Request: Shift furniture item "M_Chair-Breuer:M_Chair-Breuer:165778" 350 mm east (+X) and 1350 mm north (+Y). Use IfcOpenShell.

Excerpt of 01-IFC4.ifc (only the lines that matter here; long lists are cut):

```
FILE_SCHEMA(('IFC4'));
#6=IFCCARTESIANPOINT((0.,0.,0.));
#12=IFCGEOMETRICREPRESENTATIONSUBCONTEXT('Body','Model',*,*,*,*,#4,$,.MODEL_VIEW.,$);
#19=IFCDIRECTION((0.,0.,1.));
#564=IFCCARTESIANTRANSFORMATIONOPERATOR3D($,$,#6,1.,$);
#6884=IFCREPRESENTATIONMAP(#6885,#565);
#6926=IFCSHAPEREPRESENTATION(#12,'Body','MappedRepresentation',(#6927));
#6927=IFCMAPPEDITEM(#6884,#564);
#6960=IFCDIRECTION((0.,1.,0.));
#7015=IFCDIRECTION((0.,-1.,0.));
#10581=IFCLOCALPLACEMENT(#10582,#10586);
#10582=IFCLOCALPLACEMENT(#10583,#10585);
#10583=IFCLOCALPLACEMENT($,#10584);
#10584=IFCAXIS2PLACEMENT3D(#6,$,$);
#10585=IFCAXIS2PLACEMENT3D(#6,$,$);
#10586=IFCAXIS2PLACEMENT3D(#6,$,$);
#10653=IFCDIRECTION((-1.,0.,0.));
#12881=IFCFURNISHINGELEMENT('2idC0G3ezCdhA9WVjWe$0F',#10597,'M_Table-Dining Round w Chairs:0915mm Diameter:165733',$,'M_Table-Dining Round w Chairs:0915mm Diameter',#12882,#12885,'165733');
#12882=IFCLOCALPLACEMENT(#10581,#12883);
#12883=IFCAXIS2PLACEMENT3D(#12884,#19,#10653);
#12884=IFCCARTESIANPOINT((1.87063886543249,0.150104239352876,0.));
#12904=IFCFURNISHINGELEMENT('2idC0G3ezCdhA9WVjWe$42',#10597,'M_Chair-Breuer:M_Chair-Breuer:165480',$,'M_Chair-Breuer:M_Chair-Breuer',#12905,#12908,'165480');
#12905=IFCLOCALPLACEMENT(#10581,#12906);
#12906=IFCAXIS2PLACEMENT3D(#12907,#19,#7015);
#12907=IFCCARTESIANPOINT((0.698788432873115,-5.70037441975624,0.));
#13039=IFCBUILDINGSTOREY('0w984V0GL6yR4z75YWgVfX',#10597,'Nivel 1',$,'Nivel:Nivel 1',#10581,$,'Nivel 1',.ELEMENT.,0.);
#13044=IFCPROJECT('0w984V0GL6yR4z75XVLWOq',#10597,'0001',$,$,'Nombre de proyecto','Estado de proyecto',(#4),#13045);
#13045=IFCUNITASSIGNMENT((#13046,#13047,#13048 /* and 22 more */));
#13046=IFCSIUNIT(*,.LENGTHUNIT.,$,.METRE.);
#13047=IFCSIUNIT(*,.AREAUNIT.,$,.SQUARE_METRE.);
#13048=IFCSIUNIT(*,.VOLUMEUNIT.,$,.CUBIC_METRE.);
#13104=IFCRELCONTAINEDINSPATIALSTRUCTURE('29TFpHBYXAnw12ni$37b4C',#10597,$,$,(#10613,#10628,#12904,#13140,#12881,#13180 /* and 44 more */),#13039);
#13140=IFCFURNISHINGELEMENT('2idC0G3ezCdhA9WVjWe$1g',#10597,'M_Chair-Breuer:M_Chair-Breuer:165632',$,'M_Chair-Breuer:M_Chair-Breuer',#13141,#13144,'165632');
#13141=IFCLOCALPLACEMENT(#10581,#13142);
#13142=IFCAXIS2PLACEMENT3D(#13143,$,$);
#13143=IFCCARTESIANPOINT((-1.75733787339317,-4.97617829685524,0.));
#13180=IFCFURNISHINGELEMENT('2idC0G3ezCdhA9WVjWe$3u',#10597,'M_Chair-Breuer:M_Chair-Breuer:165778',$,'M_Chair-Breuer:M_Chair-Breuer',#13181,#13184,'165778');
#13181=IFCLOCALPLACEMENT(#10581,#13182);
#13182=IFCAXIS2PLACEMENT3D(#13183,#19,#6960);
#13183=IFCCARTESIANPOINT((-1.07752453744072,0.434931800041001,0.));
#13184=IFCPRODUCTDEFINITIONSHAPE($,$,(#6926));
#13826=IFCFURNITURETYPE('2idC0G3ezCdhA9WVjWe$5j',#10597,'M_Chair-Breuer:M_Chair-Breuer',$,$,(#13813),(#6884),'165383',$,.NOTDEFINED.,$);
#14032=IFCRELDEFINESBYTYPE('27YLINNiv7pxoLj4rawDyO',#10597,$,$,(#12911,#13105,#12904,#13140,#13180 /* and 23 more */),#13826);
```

```python
import ifcopenshell
import ifcopenshell.api.geometry
import ifcopenshell.util.placement

model = ifcopenshell.open("01-IFC4.ifc")

item = model.by_guid("2idC0G3ezCdhA9WVjWe$3u")
matrix = ifcopenshell.util.placement.get_local_placement(item.ObjectPlacement)
matrix[0, 3] += 0.35
matrix[1, 3] += 1.35
ifcopenshell.api.geometry.edit_object_placement(model, product=item, matrix=matrix, is_si=False)

print(ifcopenshell.util.placement.get_local_placement(item.ObjectPlacement).round(3) + 0.0)

model.write("01-IFC4_rev.ifc")
```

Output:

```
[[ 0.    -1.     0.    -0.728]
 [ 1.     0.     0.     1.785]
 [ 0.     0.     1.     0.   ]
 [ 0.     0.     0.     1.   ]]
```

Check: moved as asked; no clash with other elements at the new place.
